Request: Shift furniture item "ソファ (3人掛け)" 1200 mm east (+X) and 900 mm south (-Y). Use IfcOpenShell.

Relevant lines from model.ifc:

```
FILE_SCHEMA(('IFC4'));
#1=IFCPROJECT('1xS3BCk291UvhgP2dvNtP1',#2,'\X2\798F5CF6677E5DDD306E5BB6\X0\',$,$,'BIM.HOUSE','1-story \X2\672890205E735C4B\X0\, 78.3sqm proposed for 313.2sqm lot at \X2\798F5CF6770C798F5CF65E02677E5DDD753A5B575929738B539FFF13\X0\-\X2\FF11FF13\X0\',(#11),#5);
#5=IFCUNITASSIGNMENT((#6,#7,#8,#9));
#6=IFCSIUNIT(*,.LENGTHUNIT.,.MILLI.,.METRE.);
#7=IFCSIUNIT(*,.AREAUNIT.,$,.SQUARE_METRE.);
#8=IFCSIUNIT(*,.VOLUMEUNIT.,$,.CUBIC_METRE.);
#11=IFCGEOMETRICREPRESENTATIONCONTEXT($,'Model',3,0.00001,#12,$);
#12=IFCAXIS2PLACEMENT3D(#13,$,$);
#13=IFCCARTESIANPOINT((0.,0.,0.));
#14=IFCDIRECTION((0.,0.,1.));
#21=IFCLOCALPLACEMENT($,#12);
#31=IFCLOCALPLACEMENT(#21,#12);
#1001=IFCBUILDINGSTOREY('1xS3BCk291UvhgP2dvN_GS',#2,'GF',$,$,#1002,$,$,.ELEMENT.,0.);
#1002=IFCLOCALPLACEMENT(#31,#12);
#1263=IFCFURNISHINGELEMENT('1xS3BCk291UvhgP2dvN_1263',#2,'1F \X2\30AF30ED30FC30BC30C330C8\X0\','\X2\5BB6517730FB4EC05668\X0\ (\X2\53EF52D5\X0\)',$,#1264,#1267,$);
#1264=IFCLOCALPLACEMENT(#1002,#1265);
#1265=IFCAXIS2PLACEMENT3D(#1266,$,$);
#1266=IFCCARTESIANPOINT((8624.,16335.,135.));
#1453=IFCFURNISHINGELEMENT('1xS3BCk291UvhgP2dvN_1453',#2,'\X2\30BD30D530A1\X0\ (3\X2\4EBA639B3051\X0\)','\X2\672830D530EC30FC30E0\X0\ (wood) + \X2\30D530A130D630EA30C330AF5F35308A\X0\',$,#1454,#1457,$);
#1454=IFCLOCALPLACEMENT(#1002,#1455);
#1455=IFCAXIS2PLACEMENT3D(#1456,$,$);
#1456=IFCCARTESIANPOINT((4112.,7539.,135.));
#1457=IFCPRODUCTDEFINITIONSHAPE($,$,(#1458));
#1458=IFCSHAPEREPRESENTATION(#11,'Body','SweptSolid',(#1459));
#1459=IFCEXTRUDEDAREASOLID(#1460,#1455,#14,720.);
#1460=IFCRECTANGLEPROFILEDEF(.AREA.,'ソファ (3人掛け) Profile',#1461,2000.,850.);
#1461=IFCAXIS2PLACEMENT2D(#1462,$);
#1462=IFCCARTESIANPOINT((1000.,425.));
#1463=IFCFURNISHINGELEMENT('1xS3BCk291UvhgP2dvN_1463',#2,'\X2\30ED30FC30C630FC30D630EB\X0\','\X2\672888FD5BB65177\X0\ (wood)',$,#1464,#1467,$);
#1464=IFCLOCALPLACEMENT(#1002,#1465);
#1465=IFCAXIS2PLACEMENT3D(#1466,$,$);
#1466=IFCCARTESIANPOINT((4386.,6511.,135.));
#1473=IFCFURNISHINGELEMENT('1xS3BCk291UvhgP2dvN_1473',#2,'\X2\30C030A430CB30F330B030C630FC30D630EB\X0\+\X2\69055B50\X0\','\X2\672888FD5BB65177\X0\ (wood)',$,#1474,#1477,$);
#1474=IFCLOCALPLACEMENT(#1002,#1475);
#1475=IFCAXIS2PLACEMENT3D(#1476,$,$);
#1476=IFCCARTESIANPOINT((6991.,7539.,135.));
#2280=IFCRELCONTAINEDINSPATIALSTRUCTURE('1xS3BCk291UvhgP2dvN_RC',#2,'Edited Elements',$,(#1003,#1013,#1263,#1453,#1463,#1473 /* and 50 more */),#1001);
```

```python
import ifcopenshell
import ifcopenshell.api.geometry
import ifcopenshell.util.placement
import ifcopenshell.util.unit

model = ifcopenshell.open("model.ifc")
unit_scale = ifcopenshell.util.unit.calculate_unit_scale(model)

item = model.by_guid("1xS3BCk291UvhgP2dvN_1453")
matrix = ifcopenshell.util.placement.get_local_placement(item.ObjectPlacement)
matrix[0, 3] += 1.2 / unit_scale
matrix[1, 3] -= 0.9 / unit_scale
ifcopenshell.api.geometry.edit_object_placement(model, product=item, matrix=matrix, is_si=False)

print(ifcopenshell.util.placement.get_local_placement(item.ObjectPlacement).round(3) + 0.0)

model.write("model_updated.ifc")
```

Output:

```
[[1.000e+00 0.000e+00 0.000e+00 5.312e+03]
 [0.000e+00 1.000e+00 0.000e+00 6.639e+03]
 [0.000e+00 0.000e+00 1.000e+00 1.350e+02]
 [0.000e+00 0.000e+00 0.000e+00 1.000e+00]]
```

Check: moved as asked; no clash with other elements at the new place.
